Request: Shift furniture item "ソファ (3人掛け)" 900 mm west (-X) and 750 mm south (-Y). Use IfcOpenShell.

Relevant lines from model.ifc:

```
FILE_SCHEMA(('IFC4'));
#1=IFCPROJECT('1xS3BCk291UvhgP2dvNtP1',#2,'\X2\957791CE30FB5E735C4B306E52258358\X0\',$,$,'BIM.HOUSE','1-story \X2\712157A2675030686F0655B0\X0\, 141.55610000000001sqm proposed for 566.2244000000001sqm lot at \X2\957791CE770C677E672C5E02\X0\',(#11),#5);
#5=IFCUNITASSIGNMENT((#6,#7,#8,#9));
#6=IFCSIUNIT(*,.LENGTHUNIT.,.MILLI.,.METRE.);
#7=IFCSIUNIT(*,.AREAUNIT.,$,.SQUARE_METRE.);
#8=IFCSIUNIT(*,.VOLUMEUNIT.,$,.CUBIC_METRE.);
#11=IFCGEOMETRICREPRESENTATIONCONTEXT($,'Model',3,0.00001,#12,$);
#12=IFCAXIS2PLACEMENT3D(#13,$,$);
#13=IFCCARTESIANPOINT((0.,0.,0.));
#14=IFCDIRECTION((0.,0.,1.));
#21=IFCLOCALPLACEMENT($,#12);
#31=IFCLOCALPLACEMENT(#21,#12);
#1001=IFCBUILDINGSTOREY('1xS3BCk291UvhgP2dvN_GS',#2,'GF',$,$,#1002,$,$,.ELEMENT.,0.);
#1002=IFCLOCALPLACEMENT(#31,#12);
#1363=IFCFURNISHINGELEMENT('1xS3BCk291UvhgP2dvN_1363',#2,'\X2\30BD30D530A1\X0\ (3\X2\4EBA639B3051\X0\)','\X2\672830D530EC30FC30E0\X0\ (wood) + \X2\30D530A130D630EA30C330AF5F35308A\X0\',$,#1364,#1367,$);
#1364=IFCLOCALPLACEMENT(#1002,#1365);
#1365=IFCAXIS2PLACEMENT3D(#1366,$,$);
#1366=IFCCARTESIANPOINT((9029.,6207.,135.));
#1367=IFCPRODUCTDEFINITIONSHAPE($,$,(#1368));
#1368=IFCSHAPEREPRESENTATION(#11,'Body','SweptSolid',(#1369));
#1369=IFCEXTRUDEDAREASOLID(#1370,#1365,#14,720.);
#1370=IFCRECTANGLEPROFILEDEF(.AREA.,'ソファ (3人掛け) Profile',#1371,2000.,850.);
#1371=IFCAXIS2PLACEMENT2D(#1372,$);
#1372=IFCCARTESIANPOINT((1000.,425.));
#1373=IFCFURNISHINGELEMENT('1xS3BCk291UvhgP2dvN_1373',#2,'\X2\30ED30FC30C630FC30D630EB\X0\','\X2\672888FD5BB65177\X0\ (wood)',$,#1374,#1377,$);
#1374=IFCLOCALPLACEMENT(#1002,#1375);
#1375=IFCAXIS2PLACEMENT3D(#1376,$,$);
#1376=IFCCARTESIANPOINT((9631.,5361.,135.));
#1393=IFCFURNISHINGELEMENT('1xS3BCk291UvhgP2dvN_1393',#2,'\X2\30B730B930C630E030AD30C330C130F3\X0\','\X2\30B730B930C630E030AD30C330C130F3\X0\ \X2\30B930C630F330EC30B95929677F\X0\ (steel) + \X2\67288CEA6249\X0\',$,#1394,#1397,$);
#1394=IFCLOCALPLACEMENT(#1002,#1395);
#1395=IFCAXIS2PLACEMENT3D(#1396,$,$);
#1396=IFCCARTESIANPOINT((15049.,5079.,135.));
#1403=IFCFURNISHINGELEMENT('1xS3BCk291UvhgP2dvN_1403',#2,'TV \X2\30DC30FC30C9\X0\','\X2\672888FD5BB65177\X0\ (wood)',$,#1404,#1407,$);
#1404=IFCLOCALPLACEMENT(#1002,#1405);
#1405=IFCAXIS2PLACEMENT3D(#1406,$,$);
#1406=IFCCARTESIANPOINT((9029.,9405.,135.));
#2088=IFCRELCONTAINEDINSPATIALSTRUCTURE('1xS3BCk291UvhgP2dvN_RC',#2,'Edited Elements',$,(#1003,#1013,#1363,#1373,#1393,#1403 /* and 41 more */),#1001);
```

```python
import ifcopenshell
import ifcopenshell.api.geometry
import ifcopenshell.util.placement
import ifcopenshell.util.unit

model = ifcopenshell.open("model.ifc")
unit_scale = ifcopenshell.util.unit.calculate_unit_scale(model)

item = model.by_guid("1xS3BCk291UvhgP2dvN_1363")
matrix = ifcopenshell.util.placement.get_local_placement(item.ObjectPlacement)
matrix[0, 3] -= 0.9 / unit_scale
matrix[1, 3] -= 0.75 / unit_scale
ifcopenshell.api.geometry.edit_object_placement(model, product=item, matrix=matrix, is_si=False)

print(ifcopenshell.util.placement.get_local_placement(item.ObjectPlacement).round(3) + 0.0)

model.write("model_v2.ifc")
```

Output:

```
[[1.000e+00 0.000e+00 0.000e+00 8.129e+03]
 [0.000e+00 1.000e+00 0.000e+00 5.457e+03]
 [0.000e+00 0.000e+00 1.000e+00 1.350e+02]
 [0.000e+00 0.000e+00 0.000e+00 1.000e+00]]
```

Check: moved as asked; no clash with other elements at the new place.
